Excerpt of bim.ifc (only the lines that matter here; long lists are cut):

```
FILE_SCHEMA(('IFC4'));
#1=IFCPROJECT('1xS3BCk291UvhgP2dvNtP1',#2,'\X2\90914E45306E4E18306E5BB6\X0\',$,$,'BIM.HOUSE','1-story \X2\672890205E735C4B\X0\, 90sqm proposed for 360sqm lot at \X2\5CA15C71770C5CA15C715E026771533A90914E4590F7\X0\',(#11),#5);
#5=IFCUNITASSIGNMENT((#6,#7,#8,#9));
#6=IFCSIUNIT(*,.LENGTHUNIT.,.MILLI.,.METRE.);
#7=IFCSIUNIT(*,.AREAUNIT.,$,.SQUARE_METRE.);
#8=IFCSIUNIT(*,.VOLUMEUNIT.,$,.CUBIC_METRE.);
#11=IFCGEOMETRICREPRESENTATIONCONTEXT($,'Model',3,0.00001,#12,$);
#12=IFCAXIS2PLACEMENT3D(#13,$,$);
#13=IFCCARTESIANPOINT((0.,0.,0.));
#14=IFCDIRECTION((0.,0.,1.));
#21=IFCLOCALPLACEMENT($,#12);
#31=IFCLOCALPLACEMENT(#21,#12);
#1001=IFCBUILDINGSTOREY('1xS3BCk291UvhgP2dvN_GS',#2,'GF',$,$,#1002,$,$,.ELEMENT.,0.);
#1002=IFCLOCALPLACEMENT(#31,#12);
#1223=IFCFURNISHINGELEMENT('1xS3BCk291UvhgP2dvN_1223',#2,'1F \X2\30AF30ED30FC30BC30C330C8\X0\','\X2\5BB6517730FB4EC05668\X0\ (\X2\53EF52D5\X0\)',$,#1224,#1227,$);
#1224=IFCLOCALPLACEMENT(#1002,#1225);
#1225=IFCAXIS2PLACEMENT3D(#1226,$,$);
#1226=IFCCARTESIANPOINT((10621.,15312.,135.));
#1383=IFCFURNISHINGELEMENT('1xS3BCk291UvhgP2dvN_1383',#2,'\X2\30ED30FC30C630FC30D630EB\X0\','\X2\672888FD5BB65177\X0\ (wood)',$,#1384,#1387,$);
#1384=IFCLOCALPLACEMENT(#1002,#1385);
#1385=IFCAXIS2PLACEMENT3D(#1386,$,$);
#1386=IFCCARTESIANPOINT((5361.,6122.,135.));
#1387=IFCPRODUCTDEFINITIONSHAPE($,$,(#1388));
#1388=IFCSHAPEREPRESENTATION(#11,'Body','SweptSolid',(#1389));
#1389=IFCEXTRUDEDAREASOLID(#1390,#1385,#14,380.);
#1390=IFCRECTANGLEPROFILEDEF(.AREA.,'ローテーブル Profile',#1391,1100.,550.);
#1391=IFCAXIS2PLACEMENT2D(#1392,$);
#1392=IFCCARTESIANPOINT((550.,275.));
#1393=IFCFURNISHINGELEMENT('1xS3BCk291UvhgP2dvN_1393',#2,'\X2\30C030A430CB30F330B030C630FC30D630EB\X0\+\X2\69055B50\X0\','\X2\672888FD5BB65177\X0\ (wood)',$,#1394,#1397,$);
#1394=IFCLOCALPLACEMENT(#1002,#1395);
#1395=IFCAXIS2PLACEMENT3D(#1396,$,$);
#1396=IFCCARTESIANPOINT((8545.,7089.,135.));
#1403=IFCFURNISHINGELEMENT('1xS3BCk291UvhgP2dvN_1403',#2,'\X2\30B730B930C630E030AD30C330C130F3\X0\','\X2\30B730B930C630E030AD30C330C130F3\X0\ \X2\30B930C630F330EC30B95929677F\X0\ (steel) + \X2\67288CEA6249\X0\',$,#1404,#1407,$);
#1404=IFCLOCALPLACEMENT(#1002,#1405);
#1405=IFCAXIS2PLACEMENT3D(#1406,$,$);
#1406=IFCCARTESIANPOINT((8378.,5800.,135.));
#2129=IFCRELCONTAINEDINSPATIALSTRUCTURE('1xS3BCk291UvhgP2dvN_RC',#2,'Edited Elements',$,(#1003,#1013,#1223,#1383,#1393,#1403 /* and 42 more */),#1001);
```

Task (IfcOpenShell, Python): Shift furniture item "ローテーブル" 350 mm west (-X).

```python
import ifcopenshell
import ifcopenshell.api.geometry
import ifcopenshell.util.placement
import ifcopenshell.util.unit

model = ifcopenshell.open("bim.ifc")
unit_scale = ifcopenshell.util.unit.calculate_unit_scale(model)

item = model.by_guid("1xS3BCk291UvhgP2dvN_1383")
matrix = ifcopenshell.util.placement.get_local_placement(item.ObjectPlacement)
matrix[0, 3] -= 0.35 / unit_scale
ifcopenshell.api.geometry.edit_object_placement(model, product=item, matrix=matrix, is_si=False)

print(ifcopenshell.util.placement.get_local_placement(item.ObjectPlacement).round(3) + 0.0)

model.write("bim_updated.ifc")
```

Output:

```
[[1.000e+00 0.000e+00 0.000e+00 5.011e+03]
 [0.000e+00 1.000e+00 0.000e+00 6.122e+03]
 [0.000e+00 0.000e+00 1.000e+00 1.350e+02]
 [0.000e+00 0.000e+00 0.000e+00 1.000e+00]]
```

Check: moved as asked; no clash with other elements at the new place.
